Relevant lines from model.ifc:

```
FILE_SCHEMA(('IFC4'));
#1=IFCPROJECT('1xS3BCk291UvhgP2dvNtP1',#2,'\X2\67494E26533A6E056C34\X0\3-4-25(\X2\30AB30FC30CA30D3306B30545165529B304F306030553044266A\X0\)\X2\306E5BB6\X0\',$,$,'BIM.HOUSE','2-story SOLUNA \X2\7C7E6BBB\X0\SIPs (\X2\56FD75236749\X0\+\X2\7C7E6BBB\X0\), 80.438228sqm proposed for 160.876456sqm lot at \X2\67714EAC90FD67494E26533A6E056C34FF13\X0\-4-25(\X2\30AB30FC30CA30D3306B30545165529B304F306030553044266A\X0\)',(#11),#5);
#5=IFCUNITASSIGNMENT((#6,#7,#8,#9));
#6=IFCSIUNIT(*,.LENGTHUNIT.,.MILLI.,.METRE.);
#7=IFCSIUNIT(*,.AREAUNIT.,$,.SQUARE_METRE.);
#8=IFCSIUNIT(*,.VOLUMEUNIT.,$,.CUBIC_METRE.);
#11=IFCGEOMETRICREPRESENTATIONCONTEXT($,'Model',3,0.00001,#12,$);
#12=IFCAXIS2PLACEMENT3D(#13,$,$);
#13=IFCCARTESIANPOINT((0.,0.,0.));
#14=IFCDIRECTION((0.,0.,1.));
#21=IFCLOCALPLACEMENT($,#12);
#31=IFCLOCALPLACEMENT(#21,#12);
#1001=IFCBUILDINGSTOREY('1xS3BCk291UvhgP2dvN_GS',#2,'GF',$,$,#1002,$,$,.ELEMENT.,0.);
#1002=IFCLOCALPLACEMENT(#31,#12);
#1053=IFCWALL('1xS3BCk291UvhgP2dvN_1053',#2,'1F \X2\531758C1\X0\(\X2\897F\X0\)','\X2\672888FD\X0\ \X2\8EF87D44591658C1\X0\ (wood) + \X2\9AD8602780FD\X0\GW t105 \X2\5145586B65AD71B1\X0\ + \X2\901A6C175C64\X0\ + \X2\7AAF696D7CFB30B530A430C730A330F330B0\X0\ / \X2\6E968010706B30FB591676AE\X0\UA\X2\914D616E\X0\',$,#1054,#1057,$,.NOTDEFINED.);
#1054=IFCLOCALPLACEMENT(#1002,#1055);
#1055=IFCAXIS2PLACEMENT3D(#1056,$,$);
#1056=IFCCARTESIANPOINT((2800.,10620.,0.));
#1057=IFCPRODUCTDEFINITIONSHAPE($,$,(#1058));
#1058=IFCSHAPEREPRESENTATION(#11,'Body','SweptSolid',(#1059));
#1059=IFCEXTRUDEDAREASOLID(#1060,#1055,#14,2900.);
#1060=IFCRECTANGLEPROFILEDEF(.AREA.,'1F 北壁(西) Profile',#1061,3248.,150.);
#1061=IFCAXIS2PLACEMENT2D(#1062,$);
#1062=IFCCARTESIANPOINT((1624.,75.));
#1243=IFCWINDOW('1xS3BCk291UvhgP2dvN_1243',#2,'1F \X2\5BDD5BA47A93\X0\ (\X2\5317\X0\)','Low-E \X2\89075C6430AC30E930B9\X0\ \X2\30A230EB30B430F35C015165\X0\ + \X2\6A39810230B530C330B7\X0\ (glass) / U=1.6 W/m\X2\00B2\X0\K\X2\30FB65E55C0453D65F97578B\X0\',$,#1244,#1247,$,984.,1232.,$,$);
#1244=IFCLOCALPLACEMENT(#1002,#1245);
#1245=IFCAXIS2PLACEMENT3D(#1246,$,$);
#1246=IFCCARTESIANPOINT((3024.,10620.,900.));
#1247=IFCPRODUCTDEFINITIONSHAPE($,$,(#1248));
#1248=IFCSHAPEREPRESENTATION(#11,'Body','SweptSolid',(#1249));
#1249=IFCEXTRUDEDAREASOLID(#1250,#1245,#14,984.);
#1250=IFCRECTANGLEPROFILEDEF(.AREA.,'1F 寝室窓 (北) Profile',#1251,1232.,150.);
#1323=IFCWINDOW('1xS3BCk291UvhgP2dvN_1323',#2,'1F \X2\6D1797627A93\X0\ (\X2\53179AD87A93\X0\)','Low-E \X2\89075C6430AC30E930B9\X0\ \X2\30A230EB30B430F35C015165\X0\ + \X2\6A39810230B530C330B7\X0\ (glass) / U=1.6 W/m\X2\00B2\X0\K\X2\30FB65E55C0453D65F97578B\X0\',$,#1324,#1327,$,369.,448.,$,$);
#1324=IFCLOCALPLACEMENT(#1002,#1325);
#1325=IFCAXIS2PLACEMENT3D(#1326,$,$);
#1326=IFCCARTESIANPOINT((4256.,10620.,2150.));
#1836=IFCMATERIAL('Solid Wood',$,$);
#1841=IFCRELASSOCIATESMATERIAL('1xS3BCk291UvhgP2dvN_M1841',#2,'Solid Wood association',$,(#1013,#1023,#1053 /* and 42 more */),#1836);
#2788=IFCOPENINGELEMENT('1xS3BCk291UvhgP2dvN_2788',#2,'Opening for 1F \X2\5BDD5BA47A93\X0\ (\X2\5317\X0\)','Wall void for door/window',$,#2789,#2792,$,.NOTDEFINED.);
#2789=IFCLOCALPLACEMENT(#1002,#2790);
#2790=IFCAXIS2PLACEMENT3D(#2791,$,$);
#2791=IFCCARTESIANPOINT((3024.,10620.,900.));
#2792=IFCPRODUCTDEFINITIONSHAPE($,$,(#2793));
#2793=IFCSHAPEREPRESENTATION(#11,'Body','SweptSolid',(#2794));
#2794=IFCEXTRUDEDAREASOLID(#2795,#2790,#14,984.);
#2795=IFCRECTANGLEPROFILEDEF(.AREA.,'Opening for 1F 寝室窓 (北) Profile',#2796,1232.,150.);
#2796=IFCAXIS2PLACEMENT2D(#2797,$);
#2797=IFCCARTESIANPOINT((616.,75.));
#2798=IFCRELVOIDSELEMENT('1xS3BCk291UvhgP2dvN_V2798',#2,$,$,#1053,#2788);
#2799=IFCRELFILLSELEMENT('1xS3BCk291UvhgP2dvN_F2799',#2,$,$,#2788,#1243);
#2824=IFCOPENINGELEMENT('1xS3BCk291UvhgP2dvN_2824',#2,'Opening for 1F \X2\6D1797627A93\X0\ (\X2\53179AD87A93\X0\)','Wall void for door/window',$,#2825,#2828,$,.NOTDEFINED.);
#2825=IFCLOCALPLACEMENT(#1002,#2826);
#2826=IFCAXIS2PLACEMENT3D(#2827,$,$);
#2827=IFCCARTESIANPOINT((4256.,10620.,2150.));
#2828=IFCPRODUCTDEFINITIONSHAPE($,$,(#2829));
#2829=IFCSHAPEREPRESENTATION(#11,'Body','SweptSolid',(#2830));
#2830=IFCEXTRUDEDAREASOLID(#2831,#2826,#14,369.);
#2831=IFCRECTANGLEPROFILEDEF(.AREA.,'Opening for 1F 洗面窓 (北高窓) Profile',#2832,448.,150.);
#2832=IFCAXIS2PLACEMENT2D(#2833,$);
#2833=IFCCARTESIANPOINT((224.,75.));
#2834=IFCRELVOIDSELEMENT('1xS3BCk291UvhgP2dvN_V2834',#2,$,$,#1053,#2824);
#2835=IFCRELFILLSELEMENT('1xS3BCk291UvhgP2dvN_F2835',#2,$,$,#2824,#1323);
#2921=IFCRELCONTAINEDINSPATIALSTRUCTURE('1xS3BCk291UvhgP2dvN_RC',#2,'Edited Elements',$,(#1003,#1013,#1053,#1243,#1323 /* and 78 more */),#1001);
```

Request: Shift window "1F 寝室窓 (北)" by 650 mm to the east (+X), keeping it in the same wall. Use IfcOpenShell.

```python
import ifcopenshell
import ifcopenshell.api.geometry
import ifcopenshell.util.placement
import ifcopenshell.util.unit

model = ifcopenshell.open("model.ifc")
unit_scale = ifcopenshell.util.unit.calculate_unit_scale(model)

window = model.by_guid("1xS3BCk291UvhgP2dvN_1243")
opening = window.FillsVoids[0].RelatingOpeningElement
wall = opening.VoidsElements[0].RelatingBuildingElement

wall_matrix = ifcopenshell.util.placement.get_local_placement(wall.ObjectPlacement)
shift = wall_matrix[:3, 0] * 0.65 / unit_scale
before = ifcopenshell.util.placement.get_local_placement(window.ObjectPlacement)[:3, 3].copy()

# The window is not placed relative to its opening, so move both.
for product in (opening, window):
    matrix = ifcopenshell.util.placement.get_local_placement(product.ObjectPlacement)
    matrix[:3, 3] += shift
    ifcopenshell.api.geometry.edit_object_placement(model, product=product, matrix=matrix, is_si=False)

after = ifcopenshell.util.placement.get_local_placement(window.ObjectPlacement)[:3, 3]
print("window moved by", (after - before).round(3) + 0.0)

model.write("model_v2.ifc")
```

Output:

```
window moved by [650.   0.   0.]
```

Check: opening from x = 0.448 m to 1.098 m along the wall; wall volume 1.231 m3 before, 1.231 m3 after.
